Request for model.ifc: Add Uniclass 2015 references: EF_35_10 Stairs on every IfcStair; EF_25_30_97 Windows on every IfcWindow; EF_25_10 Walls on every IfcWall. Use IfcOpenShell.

First a look at what the model holds.

```python
import ifcopenshell

model = ifcopenshell.open("model.ifc")
print(model.schema)
print("classifications:", [c.Name for c in model.by_type("IfcClassification")])
for ifc_class in ("IfcDoor", "IfcRoof", "IfcStair", "IfcWall", "IfcWindow"):
    print(ifc_class, len(model.by_type(ifc_class)))
```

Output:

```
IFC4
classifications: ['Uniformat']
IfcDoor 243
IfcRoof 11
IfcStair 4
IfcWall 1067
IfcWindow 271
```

```python
import ifcopenshell
import ifcopenshell.api.classification

model = ifcopenshell.open("model.ifc")

system = ifcopenshell.api.classification.add_classification(model, classification="Uniclass 2015")

codes = {
    "IfcStair": ("EF_35_10", "Stairs"),
    "IfcWindow": ("EF_25_30_97", "Windows"),
    "IfcWall": ("EF_25_10", "Walls"),
}
for ifc_class, (code, name) in codes.items():
    products = model.by_type(ifc_class)
    ifcopenshell.api.classification.add_reference(
        model, products=products, classification=system, identification=code, name=name
    )
    print(code, len(products))

model.write("model_v2.ifc")
```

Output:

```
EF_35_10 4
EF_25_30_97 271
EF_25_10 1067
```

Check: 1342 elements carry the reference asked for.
